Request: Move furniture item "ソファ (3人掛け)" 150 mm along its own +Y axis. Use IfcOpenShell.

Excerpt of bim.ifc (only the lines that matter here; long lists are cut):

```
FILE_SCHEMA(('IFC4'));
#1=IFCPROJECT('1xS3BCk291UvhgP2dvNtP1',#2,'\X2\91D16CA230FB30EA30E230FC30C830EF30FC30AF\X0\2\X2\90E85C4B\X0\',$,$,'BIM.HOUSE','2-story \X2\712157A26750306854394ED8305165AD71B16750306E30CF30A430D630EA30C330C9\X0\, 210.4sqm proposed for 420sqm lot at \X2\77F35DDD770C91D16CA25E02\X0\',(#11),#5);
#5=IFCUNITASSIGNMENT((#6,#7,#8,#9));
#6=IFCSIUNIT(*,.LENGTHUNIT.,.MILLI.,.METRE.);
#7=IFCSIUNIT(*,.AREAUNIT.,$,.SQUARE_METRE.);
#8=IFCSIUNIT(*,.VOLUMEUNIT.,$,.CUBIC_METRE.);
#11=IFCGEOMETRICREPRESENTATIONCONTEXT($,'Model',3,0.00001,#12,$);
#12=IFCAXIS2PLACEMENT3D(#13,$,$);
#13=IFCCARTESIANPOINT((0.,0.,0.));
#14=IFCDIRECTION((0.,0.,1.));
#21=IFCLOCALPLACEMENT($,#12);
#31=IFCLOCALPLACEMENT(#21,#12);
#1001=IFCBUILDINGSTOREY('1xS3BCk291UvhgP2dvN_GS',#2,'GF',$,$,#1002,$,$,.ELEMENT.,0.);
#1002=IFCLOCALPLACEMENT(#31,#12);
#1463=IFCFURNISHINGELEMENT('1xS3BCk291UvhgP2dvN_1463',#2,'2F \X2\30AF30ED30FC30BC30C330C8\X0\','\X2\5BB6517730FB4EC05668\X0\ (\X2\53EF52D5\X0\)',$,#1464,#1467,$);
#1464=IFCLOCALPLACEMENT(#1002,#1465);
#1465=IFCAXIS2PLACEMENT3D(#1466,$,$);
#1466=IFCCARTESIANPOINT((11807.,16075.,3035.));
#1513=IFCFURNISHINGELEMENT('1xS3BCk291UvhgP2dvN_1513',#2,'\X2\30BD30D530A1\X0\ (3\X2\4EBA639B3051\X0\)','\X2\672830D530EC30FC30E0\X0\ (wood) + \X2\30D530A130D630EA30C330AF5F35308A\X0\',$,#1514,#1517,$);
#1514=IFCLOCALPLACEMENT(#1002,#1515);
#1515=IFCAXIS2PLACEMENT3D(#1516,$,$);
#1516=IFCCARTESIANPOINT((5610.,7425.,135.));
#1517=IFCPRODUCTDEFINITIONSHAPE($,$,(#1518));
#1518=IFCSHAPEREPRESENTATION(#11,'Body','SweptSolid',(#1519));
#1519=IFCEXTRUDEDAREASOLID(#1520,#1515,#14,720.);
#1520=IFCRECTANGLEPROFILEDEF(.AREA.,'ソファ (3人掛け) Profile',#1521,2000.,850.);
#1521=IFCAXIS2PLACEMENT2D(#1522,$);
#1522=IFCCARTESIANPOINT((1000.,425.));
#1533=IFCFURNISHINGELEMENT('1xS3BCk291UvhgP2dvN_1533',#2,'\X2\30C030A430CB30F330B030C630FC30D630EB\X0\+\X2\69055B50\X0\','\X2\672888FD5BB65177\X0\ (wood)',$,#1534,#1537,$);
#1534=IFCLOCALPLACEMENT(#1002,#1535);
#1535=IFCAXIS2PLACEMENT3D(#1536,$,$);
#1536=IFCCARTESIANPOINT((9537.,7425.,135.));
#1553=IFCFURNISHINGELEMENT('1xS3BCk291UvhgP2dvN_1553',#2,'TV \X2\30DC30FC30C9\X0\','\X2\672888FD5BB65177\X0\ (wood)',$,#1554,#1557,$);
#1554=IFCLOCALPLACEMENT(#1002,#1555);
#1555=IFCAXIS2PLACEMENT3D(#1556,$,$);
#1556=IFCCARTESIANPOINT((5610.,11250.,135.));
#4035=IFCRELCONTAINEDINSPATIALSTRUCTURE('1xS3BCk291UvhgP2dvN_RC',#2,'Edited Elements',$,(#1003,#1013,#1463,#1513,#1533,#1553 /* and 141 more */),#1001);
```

```python
import ifcopenshell
import ifcopenshell.api.geometry
import ifcopenshell.util.placement

model = ifcopenshell.open("bim.ifc")

item = model.by_guid("1xS3BCk291UvhgP2dvN_1513")
matrix = ifcopenshell.util.placement.get_local_placement(item.ObjectPlacement)
matrix[:3, 3] += matrix[:3, 1] * 150.0
ifcopenshell.api.geometry.edit_object_placement(model, product=item, matrix=matrix, is_si=False)

print(ifcopenshell.util.placement.get_local_placement(item.ObjectPlacement).round(3) + 0.0)

model.write("bim-out.ifc")
```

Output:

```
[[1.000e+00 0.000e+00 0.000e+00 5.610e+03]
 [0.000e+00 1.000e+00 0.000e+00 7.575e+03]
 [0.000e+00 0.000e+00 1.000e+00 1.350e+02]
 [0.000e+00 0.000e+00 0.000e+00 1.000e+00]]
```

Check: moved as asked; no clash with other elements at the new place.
